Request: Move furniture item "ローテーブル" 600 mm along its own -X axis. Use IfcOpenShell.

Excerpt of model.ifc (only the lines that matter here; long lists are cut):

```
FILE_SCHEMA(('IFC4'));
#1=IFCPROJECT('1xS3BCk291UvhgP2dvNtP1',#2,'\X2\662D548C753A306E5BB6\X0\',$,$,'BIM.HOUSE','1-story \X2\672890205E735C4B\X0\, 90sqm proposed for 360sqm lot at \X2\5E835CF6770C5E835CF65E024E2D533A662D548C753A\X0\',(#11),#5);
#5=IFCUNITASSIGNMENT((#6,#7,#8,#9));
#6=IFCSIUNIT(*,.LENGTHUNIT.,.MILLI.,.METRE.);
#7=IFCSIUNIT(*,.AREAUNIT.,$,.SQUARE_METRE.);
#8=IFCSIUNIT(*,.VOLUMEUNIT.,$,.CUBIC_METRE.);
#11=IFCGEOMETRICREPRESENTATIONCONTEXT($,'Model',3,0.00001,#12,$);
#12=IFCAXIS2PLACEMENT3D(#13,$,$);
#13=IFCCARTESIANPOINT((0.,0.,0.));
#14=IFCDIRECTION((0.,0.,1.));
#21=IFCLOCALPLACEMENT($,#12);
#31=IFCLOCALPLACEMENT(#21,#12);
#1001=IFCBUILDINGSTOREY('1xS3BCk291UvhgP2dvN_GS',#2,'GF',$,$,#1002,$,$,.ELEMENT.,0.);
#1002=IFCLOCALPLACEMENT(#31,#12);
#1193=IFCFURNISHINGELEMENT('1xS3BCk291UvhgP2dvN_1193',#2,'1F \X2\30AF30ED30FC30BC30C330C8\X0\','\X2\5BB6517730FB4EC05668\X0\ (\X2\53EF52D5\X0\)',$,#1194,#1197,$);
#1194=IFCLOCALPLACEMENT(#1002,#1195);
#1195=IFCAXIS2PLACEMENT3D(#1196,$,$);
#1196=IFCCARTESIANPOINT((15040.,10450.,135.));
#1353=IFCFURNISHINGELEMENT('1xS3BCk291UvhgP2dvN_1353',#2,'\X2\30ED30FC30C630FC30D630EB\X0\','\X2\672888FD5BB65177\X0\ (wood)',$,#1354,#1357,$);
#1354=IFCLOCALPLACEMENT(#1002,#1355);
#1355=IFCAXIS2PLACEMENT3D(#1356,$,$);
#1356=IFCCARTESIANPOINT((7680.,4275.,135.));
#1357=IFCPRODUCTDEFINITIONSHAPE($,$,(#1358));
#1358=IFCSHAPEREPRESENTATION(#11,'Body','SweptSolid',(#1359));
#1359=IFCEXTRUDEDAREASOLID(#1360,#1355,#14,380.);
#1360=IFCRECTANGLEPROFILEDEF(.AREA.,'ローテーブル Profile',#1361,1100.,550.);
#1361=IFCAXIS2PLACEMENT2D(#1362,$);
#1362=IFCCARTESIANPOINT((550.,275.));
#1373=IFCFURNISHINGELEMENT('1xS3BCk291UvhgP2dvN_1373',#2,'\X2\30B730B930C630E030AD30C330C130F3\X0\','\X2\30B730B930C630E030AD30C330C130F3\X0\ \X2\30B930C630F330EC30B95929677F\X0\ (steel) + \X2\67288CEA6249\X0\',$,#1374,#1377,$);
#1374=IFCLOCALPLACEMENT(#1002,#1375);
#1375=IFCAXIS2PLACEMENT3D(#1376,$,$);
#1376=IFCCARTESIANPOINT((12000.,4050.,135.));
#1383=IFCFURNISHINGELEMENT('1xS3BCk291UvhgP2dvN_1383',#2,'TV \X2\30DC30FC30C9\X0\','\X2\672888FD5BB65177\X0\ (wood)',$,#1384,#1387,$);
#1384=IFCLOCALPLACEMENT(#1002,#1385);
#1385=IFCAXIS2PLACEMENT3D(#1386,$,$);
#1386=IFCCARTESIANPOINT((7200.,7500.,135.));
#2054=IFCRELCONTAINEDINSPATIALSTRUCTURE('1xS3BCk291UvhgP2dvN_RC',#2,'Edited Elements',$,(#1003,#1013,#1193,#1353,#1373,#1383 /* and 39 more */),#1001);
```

```python
import ifcopenshell
import ifcopenshell.api.geometry
import ifcopenshell.util.placement
import ifcopenshell.util.unit

model = ifcopenshell.open("model.ifc")
unit_scale = ifcopenshell.util.unit.calculate_unit_scale(model)

item = model.by_guid("1xS3BCk291UvhgP2dvN_1353")
matrix = ifcopenshell.util.placement.get_local_placement(item.ObjectPlacement)
matrix[:3, 3] -= matrix[:3, 0] * 0.6 / unit_scale
ifcopenshell.api.geometry.edit_object_placement(model, product=item, matrix=matrix, is_si=False)

print(ifcopenshell.util.placement.get_local_placement(item.ObjectPlacement).round(3) + 0.0)

model.write("model_rev.ifc")
```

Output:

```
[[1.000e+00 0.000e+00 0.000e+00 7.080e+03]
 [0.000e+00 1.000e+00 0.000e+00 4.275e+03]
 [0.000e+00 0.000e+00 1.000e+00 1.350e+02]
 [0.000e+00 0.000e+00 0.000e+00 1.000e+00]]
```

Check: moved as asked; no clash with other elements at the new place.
